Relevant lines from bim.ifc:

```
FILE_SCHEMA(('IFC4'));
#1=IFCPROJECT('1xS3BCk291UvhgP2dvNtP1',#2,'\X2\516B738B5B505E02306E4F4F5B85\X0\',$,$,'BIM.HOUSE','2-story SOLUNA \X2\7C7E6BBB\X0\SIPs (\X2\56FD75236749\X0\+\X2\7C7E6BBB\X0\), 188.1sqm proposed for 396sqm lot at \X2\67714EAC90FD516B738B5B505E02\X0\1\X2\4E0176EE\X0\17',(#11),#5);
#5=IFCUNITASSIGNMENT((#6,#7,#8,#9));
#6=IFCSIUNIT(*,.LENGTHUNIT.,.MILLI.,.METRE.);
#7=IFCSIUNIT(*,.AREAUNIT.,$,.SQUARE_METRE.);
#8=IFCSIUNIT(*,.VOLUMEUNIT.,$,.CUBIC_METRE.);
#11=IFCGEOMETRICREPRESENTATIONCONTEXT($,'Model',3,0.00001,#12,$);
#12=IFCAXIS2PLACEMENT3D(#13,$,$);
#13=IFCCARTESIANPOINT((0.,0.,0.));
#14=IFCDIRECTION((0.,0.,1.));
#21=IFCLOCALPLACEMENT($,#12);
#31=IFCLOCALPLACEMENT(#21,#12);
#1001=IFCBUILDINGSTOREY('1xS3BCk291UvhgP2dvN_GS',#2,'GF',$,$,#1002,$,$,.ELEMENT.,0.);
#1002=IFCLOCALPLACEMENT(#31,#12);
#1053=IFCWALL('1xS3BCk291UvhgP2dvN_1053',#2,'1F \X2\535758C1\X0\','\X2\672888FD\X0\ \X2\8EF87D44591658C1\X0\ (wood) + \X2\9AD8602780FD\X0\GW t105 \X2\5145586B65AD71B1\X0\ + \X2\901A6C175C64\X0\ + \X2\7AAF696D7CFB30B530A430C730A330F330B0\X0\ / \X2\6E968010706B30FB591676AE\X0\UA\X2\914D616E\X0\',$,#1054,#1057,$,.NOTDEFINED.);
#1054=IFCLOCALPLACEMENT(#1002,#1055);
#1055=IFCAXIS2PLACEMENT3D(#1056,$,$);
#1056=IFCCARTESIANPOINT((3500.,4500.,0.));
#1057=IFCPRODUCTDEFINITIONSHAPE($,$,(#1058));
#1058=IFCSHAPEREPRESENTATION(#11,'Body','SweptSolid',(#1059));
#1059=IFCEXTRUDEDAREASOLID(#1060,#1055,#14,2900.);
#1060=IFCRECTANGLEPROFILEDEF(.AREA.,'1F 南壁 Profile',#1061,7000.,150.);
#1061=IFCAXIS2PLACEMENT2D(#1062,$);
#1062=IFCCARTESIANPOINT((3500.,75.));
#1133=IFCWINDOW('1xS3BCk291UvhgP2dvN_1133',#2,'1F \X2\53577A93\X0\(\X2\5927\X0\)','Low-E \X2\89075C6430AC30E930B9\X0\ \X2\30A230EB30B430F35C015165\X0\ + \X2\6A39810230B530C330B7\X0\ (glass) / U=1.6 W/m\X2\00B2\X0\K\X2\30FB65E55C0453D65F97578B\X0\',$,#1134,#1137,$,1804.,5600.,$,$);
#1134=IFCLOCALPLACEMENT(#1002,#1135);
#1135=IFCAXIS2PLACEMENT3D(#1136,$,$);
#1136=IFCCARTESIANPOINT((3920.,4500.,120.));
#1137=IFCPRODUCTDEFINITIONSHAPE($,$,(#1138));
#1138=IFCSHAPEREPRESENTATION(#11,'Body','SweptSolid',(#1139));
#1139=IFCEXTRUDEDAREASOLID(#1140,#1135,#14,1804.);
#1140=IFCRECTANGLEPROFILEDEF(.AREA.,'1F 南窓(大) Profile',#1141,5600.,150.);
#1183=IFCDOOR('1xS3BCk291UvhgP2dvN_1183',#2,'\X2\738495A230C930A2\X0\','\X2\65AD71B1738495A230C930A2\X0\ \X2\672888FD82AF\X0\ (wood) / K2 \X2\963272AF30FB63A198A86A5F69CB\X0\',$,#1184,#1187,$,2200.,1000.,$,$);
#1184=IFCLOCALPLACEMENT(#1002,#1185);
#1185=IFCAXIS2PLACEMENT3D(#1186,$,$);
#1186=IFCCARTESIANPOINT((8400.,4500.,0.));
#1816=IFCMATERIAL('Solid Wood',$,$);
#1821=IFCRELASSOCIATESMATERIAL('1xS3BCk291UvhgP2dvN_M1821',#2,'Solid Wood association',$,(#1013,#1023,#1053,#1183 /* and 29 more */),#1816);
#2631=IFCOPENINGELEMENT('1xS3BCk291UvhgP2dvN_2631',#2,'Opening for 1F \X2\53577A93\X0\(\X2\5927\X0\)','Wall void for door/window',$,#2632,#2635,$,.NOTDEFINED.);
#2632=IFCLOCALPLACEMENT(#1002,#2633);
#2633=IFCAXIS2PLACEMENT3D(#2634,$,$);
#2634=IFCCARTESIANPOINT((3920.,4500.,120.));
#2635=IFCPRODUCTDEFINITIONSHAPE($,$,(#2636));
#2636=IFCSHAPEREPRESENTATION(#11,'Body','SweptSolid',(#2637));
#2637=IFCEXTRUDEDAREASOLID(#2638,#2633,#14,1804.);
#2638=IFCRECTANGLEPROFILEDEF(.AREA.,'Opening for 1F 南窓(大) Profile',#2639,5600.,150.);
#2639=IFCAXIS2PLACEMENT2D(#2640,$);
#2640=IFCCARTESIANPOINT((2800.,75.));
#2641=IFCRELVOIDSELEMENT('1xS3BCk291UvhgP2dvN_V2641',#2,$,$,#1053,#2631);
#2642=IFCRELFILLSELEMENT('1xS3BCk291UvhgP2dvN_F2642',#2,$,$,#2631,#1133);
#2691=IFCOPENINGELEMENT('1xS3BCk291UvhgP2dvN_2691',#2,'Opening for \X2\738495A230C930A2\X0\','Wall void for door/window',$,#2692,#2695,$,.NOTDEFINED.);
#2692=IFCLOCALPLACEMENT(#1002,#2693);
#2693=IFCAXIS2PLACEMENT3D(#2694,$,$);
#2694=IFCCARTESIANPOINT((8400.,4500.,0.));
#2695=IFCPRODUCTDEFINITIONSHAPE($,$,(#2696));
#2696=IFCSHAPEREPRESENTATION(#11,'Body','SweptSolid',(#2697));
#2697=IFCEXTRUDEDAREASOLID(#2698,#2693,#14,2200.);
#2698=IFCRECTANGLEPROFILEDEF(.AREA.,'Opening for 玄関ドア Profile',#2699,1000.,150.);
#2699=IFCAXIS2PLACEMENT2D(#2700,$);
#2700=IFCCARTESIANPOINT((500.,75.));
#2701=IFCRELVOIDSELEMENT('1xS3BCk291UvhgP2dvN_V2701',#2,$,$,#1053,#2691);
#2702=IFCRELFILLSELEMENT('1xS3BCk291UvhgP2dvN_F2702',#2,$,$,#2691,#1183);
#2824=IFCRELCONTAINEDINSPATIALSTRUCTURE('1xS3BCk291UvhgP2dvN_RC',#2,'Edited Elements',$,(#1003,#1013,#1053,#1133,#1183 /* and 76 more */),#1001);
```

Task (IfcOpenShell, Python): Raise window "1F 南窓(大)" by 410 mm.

```python
import numpy as np
import ifcopenshell
import ifcopenshell.api.geometry
import ifcopenshell.util.placement
import ifcopenshell.util.unit

model = ifcopenshell.open("bim.ifc")
unit_scale = ifcopenshell.util.unit.calculate_unit_scale(model)

window = model.by_id(1133)
opening = window.FillsVoids[0].RelatingOpeningElement
dz = 0.41 / unit_scale

shift = np.array([0.0, 0.0, dz])
# The window is not placed relative to its opening, so move both.
for product in (opening, window):
    matrix = ifcopenshell.util.placement.get_local_placement(product.ObjectPlacement)
    matrix[:3, 3] += shift
    ifcopenshell.api.geometry.edit_object_placement(model, product=product, matrix=matrix, is_si=False)

print(f"moved by {dz * unit_scale:+.3f} m")

model.write("bim_rev.ifc")
```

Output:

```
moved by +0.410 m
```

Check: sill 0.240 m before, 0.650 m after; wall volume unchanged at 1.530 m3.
